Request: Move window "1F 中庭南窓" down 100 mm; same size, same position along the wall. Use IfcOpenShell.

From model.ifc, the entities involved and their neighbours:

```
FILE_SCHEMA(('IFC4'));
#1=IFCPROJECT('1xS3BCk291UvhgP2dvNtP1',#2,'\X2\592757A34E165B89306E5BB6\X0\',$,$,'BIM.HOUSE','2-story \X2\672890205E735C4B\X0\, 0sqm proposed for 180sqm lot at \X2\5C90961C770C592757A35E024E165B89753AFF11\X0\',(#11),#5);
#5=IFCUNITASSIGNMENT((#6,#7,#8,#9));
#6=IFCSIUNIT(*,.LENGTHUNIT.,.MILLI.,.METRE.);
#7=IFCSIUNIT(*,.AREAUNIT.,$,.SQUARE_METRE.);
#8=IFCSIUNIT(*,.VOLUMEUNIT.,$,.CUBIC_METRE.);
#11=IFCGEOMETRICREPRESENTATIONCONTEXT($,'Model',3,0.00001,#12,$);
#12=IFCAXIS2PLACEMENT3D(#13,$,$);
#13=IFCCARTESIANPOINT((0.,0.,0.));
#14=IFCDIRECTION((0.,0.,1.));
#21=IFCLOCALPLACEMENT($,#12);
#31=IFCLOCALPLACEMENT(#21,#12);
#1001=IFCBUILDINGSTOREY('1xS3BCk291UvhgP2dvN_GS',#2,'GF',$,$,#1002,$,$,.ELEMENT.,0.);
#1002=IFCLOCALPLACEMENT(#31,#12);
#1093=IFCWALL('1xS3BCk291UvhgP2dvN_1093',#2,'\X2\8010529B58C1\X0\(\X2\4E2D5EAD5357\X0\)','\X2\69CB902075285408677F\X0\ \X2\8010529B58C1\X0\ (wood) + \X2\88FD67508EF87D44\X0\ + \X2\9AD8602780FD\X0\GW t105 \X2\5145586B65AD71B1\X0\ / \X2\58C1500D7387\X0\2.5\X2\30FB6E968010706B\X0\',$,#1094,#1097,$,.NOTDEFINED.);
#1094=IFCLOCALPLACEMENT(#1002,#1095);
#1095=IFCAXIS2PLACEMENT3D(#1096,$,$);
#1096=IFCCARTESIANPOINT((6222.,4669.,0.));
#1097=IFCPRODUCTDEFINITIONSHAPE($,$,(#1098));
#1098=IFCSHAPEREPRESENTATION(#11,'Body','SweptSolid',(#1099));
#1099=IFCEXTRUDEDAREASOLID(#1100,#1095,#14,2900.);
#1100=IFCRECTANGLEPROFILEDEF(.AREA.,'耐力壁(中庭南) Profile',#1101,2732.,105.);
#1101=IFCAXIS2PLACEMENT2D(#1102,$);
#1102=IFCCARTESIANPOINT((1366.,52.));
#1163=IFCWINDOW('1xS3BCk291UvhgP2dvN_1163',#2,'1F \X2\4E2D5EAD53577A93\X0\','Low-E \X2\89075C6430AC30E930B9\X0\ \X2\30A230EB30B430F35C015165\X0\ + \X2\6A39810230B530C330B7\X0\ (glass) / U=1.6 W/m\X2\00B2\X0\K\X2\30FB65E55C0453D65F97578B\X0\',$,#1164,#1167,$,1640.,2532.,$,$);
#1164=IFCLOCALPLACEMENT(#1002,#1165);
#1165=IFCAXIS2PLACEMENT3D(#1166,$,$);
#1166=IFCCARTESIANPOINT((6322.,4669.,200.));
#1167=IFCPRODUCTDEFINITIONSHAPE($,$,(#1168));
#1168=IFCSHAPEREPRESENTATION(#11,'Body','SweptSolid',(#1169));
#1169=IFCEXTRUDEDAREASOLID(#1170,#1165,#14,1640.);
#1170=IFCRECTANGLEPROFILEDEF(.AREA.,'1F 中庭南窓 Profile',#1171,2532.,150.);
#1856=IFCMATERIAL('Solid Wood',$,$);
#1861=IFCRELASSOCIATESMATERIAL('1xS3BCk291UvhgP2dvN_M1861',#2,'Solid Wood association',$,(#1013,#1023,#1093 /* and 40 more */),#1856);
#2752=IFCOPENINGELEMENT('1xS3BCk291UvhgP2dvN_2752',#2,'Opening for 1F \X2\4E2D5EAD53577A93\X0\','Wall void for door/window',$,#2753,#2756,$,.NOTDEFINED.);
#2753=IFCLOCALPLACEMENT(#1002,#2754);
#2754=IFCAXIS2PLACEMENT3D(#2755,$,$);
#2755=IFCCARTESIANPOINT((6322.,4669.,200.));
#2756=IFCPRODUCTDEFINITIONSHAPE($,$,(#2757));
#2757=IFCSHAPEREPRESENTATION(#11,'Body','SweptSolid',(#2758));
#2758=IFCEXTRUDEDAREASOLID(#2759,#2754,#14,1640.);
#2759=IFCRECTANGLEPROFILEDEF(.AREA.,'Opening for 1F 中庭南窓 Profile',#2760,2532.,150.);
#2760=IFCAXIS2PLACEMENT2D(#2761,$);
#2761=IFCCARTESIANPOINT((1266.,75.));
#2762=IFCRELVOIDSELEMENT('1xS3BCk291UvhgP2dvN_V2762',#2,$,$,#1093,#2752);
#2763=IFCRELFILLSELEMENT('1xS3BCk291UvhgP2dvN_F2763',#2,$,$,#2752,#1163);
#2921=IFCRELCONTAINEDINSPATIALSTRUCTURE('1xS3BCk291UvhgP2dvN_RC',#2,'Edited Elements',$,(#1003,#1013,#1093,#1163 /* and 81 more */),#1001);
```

```python
import numpy as np
import ifcopenshell
import ifcopenshell.api.geometry
import ifcopenshell.util.placement
import ifcopenshell.util.unit

model = ifcopenshell.open("model.ifc")
unit_scale = ifcopenshell.util.unit.calculate_unit_scale(model)

window = model.by_guid("1xS3BCk291UvhgP2dvN_1163")
opening = window.FillsVoids[0].RelatingOpeningElement
dz = -100.0

shift = np.array([0.0, 0.0, dz])
# The window is not placed relative to its opening, so move both.
for product in (opening, window):
    matrix = ifcopenshell.util.placement.get_local_placement(product.ObjectPlacement)
    matrix[:3, 3] += shift
    ifcopenshell.api.geometry.edit_object_placement(model, product=product, matrix=matrix, is_si=False)

print(f"moved by {dz * unit_scale:+.3f} m")

model.write("model_rev.ifc")
```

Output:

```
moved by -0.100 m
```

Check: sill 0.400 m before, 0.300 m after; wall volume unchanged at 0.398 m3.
